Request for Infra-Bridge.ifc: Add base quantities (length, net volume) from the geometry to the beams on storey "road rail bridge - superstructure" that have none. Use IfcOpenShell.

First a look at what the model holds.

```python
import ifcopenshell
import ifcopenshell.util.element
import ifcopenshell.util.unit

model = ifcopenshell.open("Infra-Bridge.ifc")
print(model.schema)
for unit_type in ("LENGTHUNIT", "AREAUNIT", "VOLUMEUNIT"):
    print(unit_type, ifcopenshell.util.unit.calculate_unit_scale(model, unit_type))
storey = next(s for s in model.by_type("IfcBuildingStorey") if s.Name == "road rail bridge - superstructure")
beams = [e for e in ifcopenshell.util.element.get_decomposition(storey) if e.is_a("IfcBeam")]
for e in sorted(beams, key=lambda e: e.id()):
    print(e.id(), e.is_a(), e.Name, list(ifcopenshell.util.element.get_psets(e, qtos_only=True)), sep=" | ")
```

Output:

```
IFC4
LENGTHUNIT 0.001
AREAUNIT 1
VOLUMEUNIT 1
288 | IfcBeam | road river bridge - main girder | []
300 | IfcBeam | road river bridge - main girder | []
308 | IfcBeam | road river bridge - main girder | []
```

```python
import ifcopenshell
import ifcopenshell.api.pset
import ifcopenshell.geom
import ifcopenshell.util.element
import ifcopenshell.util.shape
import ifcopenshell.util.unit

model = ifcopenshell.open("Infra-Bridge.ifc")
unit_scale = ifcopenshell.util.unit.calculate_unit_scale(model)
volume_scale = ifcopenshell.util.unit.calculate_unit_scale(model, "VOLUMEUNIT")
settings = ifcopenshell.geom.settings()

storey = next(s for s in model.by_type("IfcBuildingStorey") if s.Name == "road rail bridge - superstructure")
beams = [e for e in ifcopenshell.util.element.get_decomposition(storey) if e.is_a("IfcBeam")]

for e in sorted(beams, key=lambda e: e.id()):
    if ifcopenshell.util.element.get_psets(e, qtos_only=True, should_inherit=False):
        continue
    # Geometry comes back in metres, in the element's own axes.
    shape = ifcopenshell.geom.create_shape(settings, e)
    values = {
        "Length": ifcopenshell.util.shape.get_max_xyz(shape.geometry) / unit_scale,
        "NetVolume": ifcopenshell.util.shape.get_volume(shape.geometry) / volume_scale,
    }
    qto = ifcopenshell.api.pset.add_qto(model, product=e, name="Qto_BeamBaseQuantities")
    ifcopenshell.api.pset.edit_qto(model, qto=qto, properties=values)
    print(e.id(), {k: round(v, 3) for k, v in values.items()})

model.write("Infra-Bridge-out.ifc")
```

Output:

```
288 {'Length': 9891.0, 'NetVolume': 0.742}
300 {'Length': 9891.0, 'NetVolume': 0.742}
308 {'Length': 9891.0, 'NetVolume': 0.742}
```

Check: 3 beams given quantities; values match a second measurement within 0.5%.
